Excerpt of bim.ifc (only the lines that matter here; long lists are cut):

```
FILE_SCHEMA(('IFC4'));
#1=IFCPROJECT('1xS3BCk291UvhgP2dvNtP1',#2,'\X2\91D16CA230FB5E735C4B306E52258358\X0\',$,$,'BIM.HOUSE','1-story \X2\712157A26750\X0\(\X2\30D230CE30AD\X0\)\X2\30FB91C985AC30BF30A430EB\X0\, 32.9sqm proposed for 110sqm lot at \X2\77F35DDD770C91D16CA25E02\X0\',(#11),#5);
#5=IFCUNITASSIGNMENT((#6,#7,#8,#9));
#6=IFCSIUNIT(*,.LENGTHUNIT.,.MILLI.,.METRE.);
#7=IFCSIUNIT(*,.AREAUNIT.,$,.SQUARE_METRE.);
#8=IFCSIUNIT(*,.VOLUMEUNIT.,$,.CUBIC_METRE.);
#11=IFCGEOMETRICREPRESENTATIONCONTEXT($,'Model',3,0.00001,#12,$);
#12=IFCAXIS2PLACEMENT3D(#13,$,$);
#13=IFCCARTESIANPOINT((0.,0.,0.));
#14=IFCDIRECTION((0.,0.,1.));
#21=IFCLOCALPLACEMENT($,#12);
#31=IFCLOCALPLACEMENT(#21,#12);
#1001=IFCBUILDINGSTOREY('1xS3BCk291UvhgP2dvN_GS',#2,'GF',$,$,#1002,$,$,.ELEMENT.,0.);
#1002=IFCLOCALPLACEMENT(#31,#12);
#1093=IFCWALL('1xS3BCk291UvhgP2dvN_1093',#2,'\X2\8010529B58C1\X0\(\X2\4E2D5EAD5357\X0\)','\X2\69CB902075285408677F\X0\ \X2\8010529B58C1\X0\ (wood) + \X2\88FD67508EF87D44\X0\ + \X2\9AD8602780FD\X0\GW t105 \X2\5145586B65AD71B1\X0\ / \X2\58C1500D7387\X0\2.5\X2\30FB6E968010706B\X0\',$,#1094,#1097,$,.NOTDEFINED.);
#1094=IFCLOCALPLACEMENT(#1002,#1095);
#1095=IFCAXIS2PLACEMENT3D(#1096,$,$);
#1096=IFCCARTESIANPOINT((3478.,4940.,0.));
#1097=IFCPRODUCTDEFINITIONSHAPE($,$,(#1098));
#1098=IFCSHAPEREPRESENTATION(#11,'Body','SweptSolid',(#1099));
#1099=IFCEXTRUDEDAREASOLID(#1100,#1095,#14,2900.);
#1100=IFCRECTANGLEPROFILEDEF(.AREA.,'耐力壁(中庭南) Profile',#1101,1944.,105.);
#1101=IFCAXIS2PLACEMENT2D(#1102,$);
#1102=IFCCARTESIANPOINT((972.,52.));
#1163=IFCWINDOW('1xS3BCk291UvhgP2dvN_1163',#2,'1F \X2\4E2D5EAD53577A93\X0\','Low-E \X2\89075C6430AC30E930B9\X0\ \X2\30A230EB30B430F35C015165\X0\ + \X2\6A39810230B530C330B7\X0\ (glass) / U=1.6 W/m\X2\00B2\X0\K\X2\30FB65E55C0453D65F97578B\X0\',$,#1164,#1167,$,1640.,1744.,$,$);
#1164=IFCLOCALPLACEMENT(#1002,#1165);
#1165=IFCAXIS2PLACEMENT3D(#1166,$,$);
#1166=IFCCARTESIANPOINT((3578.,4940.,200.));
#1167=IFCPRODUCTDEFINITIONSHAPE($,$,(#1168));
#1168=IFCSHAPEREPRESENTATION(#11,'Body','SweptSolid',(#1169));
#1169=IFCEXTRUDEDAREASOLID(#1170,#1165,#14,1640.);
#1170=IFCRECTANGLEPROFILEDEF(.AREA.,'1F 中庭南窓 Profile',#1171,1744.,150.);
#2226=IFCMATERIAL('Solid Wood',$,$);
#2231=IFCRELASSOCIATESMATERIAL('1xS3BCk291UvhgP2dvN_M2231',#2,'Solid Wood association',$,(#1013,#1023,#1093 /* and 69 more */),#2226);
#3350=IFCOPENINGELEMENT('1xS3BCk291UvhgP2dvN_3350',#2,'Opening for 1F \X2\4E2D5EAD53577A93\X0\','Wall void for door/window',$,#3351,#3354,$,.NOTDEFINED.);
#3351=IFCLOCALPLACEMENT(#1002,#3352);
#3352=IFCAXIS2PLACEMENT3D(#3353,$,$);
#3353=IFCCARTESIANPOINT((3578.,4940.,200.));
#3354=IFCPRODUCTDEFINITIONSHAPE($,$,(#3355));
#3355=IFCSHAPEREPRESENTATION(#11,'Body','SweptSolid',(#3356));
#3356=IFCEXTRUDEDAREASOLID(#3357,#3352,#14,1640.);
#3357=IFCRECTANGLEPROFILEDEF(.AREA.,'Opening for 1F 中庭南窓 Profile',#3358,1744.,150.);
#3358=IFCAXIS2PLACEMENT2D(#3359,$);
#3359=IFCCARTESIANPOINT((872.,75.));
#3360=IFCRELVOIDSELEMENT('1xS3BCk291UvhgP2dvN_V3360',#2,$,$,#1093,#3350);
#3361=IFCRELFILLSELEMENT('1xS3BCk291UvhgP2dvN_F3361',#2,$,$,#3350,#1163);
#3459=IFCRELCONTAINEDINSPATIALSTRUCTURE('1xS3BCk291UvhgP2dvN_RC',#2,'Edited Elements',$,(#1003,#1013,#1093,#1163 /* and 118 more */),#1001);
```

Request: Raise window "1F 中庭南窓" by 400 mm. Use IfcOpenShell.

```python
import numpy as np
import ifcopenshell
import ifcopenshell.api.geometry
import ifcopenshell.util.placement
import ifcopenshell.util.unit

model = ifcopenshell.open("bim.ifc")
unit_scale = ifcopenshell.util.unit.calculate_unit_scale(model)

window = model.by_id(1163)
opening = window.FillsVoids[0].RelatingOpeningElement
dz = 0.4 / unit_scale

shift = np.array([0.0, 0.0, dz])
# The window is not placed relative to its opening, so move both.
for product in (opening, window):
    matrix = ifcopenshell.util.placement.get_local_placement(product.ObjectPlacement)
    matrix[:3, 3] += shift
    ifcopenshell.api.geometry.edit_object_placement(model, product=product, matrix=matrix, is_si=False)

print(f"moved by {dz * unit_scale:+.3f} m")

model.write("bim_v2.ifc")
```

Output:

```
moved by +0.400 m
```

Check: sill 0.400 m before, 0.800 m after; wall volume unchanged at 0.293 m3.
